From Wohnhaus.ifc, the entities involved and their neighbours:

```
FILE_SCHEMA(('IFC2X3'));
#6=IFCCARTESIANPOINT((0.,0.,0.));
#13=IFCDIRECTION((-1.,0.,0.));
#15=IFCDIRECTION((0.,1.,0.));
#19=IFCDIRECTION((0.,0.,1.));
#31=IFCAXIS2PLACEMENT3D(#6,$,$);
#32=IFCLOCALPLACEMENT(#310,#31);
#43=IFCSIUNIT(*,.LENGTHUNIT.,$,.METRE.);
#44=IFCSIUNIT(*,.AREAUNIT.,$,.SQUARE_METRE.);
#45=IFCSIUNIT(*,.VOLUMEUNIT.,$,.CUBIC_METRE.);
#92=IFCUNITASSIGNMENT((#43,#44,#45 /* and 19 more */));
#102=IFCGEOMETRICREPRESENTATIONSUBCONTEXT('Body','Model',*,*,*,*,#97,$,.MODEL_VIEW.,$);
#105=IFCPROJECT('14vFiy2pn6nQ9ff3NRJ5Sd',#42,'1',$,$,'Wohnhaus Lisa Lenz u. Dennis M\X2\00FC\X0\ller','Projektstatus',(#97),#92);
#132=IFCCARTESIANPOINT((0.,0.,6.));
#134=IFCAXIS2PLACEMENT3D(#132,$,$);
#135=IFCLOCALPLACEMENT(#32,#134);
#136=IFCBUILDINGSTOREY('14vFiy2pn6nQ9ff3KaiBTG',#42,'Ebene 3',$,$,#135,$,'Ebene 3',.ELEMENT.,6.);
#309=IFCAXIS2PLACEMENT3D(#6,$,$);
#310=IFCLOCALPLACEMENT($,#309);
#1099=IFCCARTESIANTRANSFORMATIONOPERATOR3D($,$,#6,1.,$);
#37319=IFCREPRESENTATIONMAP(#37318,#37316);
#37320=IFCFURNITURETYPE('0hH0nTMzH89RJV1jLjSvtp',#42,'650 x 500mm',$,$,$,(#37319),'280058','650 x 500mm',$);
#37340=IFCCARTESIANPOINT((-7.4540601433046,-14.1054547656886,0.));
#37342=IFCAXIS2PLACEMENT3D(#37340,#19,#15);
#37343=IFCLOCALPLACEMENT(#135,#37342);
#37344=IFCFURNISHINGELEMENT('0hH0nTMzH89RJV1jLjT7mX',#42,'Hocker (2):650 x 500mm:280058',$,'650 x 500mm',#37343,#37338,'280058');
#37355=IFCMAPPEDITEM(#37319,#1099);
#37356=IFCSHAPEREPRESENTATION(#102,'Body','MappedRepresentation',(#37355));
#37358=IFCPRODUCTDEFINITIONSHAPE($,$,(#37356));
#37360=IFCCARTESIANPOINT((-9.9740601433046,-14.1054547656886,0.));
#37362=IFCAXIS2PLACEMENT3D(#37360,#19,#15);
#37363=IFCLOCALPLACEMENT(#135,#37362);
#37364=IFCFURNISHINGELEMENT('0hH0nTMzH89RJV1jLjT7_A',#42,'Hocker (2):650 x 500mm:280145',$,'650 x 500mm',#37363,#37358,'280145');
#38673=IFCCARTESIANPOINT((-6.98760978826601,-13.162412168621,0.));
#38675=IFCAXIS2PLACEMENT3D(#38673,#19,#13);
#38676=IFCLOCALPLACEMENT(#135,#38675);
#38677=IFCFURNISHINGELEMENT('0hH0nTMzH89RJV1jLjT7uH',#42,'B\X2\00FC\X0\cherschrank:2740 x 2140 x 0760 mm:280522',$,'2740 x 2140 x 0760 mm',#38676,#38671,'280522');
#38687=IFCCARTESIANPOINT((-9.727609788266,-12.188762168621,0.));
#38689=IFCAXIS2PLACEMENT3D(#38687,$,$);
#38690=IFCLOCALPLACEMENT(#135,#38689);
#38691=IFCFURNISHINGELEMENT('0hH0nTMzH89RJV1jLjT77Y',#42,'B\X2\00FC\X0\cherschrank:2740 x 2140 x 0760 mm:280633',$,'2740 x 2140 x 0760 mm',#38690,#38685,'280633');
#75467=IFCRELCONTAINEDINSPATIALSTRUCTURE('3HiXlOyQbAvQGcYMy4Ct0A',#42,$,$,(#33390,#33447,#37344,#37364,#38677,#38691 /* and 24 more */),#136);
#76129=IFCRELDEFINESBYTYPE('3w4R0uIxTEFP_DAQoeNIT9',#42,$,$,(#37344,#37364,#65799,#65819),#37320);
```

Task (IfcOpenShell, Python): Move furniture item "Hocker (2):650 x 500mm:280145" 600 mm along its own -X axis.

```python
import ifcopenshell
import ifcopenshell.api.geometry
import ifcopenshell.util.placement

model = ifcopenshell.open("Wohnhaus.ifc")

item = model.by_id(37364)
matrix = ifcopenshell.util.placement.get_local_placement(item.ObjectPlacement)
matrix[:3, 3] -= matrix[:3, 0] * 0.6
ifcopenshell.api.geometry.edit_object_placement(model, product=item, matrix=matrix, is_si=False)

print(ifcopenshell.util.placement.get_local_placement(item.ObjectPlacement).round(3) + 0.0)

model.write("Wohnhaus_rev.ifc")
```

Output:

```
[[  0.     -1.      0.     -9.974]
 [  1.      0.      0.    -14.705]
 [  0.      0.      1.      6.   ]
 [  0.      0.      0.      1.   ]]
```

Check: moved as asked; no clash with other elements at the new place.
